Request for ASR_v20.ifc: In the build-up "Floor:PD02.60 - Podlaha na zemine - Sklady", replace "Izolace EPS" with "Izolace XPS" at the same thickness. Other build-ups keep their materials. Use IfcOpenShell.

First a look at what the model holds.

```python
import ifcopenshell
import ifcopenshell.util.element

model = ifcopenshell.open("ASR_v20.ifc")
print(model.schema)
for layer_set in model.by_type("IfcMaterialLayerSet"):
    if layer_set.LayerSetName == "Floor:PD02.60 - Podlaha na zemine - Sklady":
        for layer in layer_set.MaterialLayers:
            print(layer.id(), layer.Material and layer.Material.Name, layer.LayerThickness, sep=" | ")
        print(len(ifcopenshell.util.element.get_elements_by_material(model, layer_set)), "elements and types use it")
print(sorted(m.Name for m in model.by_type("IfcMaterial") if m.Name)[:60])
```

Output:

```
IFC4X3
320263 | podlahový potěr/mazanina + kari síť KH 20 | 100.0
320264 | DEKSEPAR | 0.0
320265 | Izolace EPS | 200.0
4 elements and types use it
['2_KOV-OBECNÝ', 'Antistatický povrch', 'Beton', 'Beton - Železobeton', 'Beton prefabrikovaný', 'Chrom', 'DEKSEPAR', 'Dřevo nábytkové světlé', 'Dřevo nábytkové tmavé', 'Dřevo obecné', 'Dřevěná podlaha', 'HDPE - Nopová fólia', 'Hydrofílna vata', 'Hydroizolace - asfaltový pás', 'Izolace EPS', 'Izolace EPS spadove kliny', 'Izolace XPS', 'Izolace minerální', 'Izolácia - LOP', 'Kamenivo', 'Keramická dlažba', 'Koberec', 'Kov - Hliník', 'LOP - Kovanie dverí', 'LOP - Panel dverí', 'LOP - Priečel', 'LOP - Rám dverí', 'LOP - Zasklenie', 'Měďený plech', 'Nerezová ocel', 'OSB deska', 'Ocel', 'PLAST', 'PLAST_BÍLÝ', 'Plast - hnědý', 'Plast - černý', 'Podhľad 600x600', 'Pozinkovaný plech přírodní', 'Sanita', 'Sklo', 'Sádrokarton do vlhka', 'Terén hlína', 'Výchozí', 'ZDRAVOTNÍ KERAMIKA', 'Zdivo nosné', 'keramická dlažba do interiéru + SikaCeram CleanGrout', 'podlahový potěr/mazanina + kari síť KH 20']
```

```python
import ifcopenshell
import ifcopenshell.api.material

model = ifcopenshell.open("ASR_v20.ifc")

layer_set = next(s for s in model.by_type("IfcMaterialLayerSet") if s.LayerSetName == "Floor:PD02.60 - Podlaha na zemine - Sklady")
layer = next(l for l in layer_set.MaterialLayers if l.Material and l.Material.Name == "Izolace EPS")
material = next(m for m in model.by_type("IfcMaterial") if m.Name == "Izolace XPS")

# Point this one layer at the other material; renaming the old one would change it everywhere.
ifcopenshell.api.material.edit_layer(model, layer=layer, attributes={"Name": material.Name}, material=material)

print([l.Material.Name if l.Material else None for l in layer_set.MaterialLayers])

model.write("ASR_v20_rev.ifc")
```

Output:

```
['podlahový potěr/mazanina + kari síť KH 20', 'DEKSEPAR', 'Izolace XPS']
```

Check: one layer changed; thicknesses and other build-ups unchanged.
